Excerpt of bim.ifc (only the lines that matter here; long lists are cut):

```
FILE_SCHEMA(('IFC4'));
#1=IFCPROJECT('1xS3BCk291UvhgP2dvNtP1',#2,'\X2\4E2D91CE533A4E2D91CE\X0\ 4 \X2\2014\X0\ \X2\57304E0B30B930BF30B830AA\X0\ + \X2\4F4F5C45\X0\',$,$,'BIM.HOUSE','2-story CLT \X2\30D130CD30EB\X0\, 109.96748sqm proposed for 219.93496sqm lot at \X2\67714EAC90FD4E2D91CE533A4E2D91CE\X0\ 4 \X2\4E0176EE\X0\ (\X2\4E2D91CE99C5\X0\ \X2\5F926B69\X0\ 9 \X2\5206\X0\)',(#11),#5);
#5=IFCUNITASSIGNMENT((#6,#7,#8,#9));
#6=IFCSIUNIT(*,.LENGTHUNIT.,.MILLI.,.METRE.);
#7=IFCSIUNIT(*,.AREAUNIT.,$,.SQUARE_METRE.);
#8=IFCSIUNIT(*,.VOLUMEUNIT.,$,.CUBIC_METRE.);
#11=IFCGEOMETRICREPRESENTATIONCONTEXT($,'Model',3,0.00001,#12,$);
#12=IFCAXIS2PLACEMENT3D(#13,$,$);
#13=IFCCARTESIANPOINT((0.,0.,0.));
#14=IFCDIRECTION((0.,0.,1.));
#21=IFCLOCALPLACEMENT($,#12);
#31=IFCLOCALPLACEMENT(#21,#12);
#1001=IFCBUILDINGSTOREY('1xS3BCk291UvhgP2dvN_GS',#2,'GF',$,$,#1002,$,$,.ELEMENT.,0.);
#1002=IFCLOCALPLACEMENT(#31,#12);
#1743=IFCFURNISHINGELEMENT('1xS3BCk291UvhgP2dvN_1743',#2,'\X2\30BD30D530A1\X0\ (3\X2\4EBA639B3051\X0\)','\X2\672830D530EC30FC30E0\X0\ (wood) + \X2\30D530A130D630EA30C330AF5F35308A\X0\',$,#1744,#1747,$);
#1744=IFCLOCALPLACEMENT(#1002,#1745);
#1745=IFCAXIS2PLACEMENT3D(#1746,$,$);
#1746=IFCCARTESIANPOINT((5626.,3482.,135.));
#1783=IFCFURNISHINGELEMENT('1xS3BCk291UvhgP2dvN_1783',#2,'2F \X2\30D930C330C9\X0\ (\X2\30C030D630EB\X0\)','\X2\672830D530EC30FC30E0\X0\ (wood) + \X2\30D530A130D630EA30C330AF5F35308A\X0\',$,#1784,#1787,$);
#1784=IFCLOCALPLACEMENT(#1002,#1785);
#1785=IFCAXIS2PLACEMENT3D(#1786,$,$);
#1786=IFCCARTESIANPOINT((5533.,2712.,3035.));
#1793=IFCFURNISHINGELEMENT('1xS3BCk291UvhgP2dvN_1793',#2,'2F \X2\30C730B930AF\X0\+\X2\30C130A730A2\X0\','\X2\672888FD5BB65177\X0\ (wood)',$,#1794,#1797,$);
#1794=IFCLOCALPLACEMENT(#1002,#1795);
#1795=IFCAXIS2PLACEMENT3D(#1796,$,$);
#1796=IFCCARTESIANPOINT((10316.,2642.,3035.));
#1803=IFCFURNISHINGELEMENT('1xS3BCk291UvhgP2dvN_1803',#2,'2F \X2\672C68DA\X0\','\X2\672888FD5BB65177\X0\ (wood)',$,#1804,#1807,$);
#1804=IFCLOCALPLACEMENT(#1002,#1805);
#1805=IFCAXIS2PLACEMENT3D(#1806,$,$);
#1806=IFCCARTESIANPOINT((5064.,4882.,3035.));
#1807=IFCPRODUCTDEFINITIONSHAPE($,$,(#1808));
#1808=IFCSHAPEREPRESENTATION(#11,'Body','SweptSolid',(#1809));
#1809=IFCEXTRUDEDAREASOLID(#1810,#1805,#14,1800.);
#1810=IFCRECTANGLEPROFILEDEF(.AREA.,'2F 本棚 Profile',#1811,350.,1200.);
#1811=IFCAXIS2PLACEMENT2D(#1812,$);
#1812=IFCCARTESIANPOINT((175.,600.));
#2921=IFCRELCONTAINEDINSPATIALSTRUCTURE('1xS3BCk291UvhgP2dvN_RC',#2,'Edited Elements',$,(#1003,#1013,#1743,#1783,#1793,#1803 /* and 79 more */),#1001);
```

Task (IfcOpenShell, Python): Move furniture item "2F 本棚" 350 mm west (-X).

```python
import ifcopenshell
import ifcopenshell.api.geometry
import ifcopenshell.util.placement

model = ifcopenshell.open("bim.ifc")

item = model.by_guid("1xS3BCk291UvhgP2dvN_1803")
matrix = ifcopenshell.util.placement.get_local_placement(item.ObjectPlacement)
matrix[0, 3] -= 350.0
ifcopenshell.api.geometry.edit_object_placement(model, product=item, matrix=matrix, is_si=False)

print(ifcopenshell.util.placement.get_local_placement(item.ObjectPlacement).round(3) + 0.0)

model.write("bim_updated.ifc")
```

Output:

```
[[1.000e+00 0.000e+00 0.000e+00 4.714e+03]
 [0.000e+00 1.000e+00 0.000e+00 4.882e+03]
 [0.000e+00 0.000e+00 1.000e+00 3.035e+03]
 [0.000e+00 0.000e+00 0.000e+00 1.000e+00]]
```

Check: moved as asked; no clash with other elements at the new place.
